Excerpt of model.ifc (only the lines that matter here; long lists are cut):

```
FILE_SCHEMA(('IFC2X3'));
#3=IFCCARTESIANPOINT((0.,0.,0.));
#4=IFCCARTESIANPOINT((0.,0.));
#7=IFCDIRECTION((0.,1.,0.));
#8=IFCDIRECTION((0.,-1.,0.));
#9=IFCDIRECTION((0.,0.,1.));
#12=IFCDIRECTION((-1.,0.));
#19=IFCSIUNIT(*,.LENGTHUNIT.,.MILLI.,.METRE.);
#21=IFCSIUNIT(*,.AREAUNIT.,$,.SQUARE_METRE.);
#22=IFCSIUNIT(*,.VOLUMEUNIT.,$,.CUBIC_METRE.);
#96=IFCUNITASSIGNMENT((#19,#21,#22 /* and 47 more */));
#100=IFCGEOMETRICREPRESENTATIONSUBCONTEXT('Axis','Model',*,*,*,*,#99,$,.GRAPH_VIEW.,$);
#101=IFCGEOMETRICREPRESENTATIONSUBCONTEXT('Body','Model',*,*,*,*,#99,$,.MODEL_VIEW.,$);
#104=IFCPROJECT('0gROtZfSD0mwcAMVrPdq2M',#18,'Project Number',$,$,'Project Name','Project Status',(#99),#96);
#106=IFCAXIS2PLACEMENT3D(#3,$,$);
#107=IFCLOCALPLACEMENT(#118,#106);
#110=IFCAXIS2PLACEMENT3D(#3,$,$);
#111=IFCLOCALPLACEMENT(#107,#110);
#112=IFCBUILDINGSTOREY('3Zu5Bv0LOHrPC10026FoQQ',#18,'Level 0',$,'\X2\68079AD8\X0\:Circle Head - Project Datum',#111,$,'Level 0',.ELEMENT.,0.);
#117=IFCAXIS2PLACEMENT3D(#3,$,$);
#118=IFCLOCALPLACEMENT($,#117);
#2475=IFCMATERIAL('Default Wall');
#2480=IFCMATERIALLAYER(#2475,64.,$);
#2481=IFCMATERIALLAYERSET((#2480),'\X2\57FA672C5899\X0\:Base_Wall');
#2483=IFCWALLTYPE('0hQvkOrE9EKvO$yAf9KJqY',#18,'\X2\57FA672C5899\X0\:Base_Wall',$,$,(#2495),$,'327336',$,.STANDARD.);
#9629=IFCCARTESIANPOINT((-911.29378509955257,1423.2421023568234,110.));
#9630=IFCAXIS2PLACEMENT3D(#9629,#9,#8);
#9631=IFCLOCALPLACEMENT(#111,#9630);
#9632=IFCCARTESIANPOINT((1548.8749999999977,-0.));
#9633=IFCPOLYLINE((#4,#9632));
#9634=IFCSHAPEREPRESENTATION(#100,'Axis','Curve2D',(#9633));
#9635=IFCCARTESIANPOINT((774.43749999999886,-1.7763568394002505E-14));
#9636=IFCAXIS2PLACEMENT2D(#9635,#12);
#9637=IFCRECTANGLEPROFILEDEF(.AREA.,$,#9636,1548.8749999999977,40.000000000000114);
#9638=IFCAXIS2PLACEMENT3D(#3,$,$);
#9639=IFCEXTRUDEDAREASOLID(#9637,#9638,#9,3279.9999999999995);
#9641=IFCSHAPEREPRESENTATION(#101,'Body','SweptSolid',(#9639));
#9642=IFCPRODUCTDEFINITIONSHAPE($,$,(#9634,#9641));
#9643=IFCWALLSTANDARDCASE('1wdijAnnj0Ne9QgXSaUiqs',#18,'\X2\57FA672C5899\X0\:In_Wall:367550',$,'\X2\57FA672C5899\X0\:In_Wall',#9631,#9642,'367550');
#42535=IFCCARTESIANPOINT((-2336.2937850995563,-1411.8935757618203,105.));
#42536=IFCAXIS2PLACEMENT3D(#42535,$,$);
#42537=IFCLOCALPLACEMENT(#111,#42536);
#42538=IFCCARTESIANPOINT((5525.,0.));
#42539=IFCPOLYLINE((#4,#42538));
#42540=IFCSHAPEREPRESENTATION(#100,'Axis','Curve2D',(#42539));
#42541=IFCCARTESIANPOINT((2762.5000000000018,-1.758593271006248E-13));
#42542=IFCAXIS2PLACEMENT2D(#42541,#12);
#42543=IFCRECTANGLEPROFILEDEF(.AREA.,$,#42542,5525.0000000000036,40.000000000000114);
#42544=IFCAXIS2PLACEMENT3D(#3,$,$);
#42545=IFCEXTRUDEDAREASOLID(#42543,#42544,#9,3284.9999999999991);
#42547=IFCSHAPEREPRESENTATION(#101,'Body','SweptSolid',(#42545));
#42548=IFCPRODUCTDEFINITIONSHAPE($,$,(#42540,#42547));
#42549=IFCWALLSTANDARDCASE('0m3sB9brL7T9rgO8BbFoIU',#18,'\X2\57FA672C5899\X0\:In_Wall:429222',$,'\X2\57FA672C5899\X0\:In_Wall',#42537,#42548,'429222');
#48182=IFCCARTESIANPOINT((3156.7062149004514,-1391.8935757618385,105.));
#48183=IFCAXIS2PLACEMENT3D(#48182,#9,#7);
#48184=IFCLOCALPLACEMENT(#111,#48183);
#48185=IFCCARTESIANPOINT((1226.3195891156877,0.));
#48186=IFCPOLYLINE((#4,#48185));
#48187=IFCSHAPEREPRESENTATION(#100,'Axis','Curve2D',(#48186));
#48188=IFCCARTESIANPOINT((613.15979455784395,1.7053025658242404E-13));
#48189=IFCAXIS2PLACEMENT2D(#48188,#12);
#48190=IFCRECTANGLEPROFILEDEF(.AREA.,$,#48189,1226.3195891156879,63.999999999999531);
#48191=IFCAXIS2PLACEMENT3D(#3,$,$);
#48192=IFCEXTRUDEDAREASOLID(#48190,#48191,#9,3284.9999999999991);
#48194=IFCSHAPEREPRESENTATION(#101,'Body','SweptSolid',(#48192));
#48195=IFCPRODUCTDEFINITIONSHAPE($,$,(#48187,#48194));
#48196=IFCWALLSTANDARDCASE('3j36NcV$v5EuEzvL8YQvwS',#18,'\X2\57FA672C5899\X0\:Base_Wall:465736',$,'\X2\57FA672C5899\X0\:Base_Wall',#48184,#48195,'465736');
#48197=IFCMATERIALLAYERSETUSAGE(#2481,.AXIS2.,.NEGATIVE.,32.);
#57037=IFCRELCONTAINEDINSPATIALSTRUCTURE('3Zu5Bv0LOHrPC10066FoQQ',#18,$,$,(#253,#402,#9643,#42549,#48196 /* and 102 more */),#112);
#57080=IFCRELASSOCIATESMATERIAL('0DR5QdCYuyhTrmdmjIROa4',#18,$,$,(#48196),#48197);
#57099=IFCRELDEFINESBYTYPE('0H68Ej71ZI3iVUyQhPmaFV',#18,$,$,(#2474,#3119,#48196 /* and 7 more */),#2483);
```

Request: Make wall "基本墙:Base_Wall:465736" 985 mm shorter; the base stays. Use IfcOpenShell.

```python
import ifcopenshell
import ifcopenshell.geom
import ifcopenshell.util.representation
import ifcopenshell.util.shape
import ifcopenshell.util.unit

model = ifcopenshell.open("model.ifc")
unit_scale = ifcopenshell.util.unit.calculate_unit_scale(model)
settings = ifcopenshell.geom.settings()


def volume(element):
    """Net volume in cubic metres, openings subtracted."""
    shape = ifcopenshell.geom.create_shape(settings, element)
    return ifcopenshell.util.shape.get_volume(shape.geometry)


wall = model.by_id(48196)
before = volume(wall)

body = ifcopenshell.util.representation.get_representation(wall, "Model", "Body")
solid = body.Items[0]
old_height = solid.Depth
solid.Depth -= 0.985 / unit_scale
after = volume(wall)

print(f"height {old_height:g} -> {solid.Depth:g}, volume {before:.3f} -> {after:.3f} m3")

model.write("model-out.ifc")
```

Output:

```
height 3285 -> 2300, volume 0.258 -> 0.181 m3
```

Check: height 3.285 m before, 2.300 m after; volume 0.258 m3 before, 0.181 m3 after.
